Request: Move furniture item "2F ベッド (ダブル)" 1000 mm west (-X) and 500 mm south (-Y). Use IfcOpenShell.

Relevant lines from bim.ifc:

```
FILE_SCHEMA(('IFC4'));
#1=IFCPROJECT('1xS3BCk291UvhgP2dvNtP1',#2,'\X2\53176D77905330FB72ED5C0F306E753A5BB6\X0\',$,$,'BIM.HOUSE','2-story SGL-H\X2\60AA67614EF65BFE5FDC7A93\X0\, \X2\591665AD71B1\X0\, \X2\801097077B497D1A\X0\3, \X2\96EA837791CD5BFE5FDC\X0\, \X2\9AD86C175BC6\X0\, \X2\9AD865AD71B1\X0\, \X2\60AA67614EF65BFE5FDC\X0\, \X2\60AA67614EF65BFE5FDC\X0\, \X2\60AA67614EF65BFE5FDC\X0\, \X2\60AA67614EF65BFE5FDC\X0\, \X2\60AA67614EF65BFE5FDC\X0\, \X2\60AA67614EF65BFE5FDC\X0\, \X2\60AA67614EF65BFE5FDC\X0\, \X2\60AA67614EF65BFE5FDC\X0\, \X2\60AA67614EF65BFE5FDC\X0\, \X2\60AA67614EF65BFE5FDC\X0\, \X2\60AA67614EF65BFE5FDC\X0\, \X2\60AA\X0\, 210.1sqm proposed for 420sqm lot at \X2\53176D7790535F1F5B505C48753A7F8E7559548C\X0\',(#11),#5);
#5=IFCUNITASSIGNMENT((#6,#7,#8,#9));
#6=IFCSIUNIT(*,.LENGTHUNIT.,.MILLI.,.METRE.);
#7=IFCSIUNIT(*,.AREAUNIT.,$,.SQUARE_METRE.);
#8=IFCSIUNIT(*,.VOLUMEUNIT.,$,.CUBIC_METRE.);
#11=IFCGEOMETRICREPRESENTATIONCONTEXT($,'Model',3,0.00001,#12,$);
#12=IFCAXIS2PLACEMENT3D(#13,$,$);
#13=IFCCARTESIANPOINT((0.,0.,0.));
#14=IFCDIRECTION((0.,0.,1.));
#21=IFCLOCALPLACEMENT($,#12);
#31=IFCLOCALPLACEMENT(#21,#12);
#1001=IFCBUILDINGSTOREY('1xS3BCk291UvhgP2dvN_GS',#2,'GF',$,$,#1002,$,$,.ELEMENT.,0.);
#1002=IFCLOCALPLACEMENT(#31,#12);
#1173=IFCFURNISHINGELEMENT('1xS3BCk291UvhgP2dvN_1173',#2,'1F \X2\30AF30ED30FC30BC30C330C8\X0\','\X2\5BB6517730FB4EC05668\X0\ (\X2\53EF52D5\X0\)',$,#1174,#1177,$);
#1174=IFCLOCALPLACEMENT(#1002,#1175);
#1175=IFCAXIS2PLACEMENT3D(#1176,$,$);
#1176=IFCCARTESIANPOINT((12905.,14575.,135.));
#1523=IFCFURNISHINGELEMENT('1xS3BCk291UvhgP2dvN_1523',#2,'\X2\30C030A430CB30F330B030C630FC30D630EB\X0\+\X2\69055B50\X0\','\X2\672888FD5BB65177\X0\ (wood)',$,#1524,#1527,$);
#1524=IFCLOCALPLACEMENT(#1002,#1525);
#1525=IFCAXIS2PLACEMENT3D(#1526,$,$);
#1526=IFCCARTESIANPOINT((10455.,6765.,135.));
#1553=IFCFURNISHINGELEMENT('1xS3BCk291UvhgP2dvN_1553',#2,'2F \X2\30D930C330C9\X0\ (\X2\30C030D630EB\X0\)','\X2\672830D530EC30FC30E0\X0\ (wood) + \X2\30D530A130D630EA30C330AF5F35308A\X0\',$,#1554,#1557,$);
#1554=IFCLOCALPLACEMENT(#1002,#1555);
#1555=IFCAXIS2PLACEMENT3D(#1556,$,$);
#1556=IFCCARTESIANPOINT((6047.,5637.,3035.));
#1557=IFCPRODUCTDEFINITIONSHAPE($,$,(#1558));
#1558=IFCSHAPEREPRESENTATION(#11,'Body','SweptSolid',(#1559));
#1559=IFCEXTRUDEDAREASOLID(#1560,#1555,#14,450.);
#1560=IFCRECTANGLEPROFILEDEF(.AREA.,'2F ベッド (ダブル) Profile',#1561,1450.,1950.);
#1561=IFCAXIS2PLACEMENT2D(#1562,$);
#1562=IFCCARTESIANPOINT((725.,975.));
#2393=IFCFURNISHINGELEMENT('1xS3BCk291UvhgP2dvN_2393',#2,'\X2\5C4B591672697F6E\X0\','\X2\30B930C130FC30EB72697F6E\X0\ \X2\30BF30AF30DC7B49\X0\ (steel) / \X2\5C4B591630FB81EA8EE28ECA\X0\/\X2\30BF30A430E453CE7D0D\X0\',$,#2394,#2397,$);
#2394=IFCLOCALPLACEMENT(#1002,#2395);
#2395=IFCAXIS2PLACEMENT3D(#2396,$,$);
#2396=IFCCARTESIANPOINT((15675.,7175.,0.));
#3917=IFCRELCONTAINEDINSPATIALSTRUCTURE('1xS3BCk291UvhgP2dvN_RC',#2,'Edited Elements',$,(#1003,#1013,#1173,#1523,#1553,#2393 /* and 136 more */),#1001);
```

```python
import ifcopenshell
import ifcopenshell.api.geometry
import ifcopenshell.util.placement
import ifcopenshell.util.unit

model = ifcopenshell.open("bim.ifc")
unit_scale = ifcopenshell.util.unit.calculate_unit_scale(model)

item = model.by_guid("1xS3BCk291UvhgP2dvN_1553")
matrix = ifcopenshell.util.placement.get_local_placement(item.ObjectPlacement)
matrix[0, 3] -= 1 / unit_scale
matrix[1, 3] -= 0.5 / unit_scale
ifcopenshell.api.geometry.edit_object_placement(model, product=item, matrix=matrix, is_si=False)

print(ifcopenshell.util.placement.get_local_placement(item.ObjectPlacement).round(3) + 0.0)

model.write("bim_edited.ifc")
```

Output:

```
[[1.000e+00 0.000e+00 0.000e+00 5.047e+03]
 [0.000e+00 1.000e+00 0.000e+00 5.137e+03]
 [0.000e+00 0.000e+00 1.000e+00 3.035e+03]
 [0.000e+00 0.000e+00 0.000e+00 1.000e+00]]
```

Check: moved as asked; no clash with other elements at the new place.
